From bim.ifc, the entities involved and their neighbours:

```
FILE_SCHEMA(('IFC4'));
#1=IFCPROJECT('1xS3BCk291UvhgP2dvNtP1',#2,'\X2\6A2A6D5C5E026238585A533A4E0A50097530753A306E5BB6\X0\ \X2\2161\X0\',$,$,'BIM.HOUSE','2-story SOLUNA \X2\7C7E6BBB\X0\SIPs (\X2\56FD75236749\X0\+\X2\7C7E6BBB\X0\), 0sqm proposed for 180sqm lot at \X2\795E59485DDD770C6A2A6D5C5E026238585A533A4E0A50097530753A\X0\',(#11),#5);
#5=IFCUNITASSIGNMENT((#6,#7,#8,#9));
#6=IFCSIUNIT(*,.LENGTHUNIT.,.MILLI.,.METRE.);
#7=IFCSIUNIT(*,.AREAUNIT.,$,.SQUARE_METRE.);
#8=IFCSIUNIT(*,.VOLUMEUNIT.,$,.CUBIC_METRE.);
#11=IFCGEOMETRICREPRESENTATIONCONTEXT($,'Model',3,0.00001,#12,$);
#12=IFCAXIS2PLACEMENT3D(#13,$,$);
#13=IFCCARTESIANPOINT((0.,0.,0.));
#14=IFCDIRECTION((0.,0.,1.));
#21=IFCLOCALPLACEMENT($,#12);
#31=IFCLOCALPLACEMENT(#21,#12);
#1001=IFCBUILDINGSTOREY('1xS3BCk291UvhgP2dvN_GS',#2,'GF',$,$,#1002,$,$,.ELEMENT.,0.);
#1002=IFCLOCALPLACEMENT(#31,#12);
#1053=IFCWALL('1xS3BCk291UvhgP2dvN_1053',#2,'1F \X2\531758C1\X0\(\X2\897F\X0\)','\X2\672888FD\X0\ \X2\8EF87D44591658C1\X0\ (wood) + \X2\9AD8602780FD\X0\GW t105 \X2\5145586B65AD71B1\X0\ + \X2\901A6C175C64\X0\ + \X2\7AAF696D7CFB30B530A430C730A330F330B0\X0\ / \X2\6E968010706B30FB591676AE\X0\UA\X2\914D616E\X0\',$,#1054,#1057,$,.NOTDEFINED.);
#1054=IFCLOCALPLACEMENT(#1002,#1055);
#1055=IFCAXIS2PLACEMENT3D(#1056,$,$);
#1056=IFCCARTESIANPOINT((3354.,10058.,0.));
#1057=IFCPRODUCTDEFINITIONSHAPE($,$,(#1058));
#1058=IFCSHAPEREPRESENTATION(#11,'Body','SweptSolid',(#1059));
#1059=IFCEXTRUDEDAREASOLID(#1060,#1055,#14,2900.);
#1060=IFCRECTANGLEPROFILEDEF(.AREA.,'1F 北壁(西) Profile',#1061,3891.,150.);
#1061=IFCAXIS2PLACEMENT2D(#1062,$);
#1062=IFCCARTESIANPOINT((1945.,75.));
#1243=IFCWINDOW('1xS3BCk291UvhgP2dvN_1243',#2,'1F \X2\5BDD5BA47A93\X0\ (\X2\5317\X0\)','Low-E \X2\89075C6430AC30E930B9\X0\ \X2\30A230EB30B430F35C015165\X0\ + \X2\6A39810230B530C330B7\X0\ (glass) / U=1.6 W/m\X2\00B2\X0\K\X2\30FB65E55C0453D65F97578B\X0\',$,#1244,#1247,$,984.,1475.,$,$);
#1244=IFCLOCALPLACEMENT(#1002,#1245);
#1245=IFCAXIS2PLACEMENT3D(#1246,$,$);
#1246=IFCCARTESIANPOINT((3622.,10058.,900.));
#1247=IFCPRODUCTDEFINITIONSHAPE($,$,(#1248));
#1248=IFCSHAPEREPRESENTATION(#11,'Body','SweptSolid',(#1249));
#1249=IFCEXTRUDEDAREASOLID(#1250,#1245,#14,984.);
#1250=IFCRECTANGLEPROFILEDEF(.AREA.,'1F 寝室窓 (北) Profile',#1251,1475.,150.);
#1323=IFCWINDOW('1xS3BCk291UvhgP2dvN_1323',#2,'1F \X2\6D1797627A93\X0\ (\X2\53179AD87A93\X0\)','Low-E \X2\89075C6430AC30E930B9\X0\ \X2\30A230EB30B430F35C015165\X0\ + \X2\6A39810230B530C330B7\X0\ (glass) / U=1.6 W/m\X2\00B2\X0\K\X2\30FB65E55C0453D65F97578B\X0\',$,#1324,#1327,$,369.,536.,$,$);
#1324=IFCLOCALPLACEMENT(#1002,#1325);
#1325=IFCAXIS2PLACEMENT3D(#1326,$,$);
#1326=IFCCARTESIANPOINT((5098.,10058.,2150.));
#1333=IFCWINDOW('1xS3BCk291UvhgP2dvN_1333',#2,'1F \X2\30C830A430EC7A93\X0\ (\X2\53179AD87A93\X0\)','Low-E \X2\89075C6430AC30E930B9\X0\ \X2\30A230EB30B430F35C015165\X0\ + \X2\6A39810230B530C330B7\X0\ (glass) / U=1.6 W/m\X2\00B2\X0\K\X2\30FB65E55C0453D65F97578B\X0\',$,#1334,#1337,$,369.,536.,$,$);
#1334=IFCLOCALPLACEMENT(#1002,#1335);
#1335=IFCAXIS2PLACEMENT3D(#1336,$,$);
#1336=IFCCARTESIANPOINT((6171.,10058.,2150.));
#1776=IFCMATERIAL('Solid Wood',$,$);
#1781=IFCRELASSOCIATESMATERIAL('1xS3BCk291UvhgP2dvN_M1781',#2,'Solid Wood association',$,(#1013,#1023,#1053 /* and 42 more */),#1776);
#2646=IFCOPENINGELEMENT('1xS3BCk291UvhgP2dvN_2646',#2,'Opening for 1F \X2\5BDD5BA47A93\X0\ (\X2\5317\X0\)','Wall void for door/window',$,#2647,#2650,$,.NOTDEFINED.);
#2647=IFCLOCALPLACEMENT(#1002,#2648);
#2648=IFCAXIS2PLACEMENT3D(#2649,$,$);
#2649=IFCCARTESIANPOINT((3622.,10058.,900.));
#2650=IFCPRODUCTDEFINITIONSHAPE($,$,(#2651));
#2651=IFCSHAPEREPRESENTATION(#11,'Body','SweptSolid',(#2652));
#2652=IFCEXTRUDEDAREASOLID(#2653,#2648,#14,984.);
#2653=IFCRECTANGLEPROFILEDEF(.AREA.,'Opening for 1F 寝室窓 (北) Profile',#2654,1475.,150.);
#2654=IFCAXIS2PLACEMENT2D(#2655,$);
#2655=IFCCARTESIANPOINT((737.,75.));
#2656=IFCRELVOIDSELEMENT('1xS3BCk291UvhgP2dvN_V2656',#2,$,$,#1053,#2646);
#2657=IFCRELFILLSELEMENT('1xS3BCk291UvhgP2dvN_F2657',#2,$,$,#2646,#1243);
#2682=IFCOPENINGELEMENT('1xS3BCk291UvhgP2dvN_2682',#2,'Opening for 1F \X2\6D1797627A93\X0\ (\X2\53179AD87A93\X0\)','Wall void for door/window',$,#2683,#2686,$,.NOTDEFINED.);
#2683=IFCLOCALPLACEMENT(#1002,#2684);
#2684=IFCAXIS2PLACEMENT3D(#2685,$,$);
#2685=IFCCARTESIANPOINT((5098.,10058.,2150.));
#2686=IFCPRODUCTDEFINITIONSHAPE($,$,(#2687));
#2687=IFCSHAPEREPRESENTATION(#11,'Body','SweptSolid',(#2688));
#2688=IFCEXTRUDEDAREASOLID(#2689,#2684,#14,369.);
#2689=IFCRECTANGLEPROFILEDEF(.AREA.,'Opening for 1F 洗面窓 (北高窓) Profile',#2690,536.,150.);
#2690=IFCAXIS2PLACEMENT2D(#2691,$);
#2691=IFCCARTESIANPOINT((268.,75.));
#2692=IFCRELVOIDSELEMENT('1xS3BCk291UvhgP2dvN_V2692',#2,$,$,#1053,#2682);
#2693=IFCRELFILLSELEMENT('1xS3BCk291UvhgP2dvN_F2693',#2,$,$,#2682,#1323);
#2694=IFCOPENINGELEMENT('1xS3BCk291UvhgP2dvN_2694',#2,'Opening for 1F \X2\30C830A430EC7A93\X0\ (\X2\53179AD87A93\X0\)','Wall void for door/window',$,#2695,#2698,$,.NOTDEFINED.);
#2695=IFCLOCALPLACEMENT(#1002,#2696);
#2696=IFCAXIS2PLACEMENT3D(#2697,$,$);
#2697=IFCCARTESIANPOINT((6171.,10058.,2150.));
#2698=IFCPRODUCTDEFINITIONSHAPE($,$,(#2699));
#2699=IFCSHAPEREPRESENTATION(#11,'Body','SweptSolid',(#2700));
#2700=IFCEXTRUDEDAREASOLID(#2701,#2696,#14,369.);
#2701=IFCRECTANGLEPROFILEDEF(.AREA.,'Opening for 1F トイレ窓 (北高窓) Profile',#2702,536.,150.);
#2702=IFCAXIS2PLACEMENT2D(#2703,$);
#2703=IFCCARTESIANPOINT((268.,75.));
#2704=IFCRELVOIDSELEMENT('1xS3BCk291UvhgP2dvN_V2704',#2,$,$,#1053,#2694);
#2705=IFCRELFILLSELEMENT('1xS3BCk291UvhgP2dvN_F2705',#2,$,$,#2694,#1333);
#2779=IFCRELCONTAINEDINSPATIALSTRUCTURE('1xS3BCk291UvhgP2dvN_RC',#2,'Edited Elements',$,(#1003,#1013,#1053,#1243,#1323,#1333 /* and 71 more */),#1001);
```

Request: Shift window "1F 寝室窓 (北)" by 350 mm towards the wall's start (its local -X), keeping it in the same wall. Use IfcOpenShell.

```python
import ifcopenshell
import ifcopenshell.api.geometry
import ifcopenshell.util.placement
import ifcopenshell.util.unit

model = ifcopenshell.open("bim.ifc")
unit_scale = ifcopenshell.util.unit.calculate_unit_scale(model)

window = model.by_guid("1xS3BCk291UvhgP2dvN_1243")
opening = window.FillsVoids[0].RelatingOpeningElement
wall = opening.VoidsElements[0].RelatingBuildingElement

wall_matrix = ifcopenshell.util.placement.get_local_placement(wall.ObjectPlacement)
shift = wall_matrix[:3, 0] * -0.35 / unit_scale
before = ifcopenshell.util.placement.get_local_placement(window.ObjectPlacement)[:3, 3].copy()

# The window is not placed relative to its opening, so move both.
for product in (opening, window):
    matrix = ifcopenshell.util.placement.get_local_placement(product.ObjectPlacement)
    matrix[:3, 3] += shift
    ifcopenshell.api.geometry.edit_object_placement(model, product=product, matrix=matrix, is_si=False)

after = ifcopenshell.util.placement.get_local_placement(window.ObjectPlacement)[:3, 3]
print("window moved by", (after - before).round(3) + 0.0)

model.write("bim-out.ifc")
```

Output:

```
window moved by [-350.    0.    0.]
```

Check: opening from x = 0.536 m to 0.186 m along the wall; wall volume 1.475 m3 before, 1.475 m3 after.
